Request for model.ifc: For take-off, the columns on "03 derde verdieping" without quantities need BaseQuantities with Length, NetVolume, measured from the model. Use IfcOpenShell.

First a look at what the model holds.

```python
import ifcopenshell
import ifcopenshell.util.element
import ifcopenshell.util.unit

model = ifcopenshell.open("model.ifc")
print(model.schema)
for unit_type in ("LENGTHUNIT", "AREAUNIT", "VOLUMEUNIT"):
    print(unit_type, ifcopenshell.util.unit.calculate_unit_scale(model, unit_type))
storey = next(s for s in model.by_type("IfcBuildingStorey") if s.Name == "03 derde verdieping")
columns = [e for e in ifcopenshell.util.element.get_decomposition(storey) if e.is_a("IfcColumn")]
for e in sorted(columns, key=lambda e: e.id()):
    print(e.id(), e.is_a(), e.Name, list(ifcopenshell.util.element.get_psets(e, qtos_only=True)), sep=" | ")
```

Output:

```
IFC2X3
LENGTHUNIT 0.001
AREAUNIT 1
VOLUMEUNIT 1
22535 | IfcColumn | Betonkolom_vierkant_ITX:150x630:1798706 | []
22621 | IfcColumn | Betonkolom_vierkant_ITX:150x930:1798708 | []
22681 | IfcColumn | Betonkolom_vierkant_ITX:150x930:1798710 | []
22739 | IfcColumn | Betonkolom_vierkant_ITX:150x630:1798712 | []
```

```python
import ifcopenshell
import ifcopenshell.api.pset
import ifcopenshell.geom
import ifcopenshell.util.element
import ifcopenshell.util.shape
import ifcopenshell.util.unit

model = ifcopenshell.open("model.ifc")
unit_scale = ifcopenshell.util.unit.calculate_unit_scale(model)
volume_scale = ifcopenshell.util.unit.calculate_unit_scale(model, "VOLUMEUNIT")
settings = ifcopenshell.geom.settings()

storey = next(s for s in model.by_type("IfcBuildingStorey") if s.Name == "03 derde verdieping")
columns = [e for e in ifcopenshell.util.element.get_decomposition(storey) if e.is_a("IfcColumn")]

for e in sorted(columns, key=lambda e: e.id()):
    if ifcopenshell.util.element.get_psets(e, qtos_only=True, should_inherit=False):
        continue
    # Geometry comes back in metres, in the element's own axes.
    shape = ifcopenshell.geom.create_shape(settings, e)
    values = {
        "Length": ifcopenshell.util.shape.get_z(shape.geometry) / unit_scale,
        "NetVolume": ifcopenshell.util.shape.get_volume(shape.geometry) / volume_scale,
    }
    qto = ifcopenshell.api.pset.add_qto(model, product=e, name="BaseQuantities")
    ifcopenshell.api.pset.edit_qto(model, qto=qto, properties=values)
    print(e.id(), {k: round(v, 3) for k, v in values.items()})

model.write("model-out.ifc")
```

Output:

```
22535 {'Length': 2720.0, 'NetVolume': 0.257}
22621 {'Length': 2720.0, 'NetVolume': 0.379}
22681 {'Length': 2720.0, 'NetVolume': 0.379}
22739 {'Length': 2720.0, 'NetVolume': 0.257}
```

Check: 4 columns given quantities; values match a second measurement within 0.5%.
